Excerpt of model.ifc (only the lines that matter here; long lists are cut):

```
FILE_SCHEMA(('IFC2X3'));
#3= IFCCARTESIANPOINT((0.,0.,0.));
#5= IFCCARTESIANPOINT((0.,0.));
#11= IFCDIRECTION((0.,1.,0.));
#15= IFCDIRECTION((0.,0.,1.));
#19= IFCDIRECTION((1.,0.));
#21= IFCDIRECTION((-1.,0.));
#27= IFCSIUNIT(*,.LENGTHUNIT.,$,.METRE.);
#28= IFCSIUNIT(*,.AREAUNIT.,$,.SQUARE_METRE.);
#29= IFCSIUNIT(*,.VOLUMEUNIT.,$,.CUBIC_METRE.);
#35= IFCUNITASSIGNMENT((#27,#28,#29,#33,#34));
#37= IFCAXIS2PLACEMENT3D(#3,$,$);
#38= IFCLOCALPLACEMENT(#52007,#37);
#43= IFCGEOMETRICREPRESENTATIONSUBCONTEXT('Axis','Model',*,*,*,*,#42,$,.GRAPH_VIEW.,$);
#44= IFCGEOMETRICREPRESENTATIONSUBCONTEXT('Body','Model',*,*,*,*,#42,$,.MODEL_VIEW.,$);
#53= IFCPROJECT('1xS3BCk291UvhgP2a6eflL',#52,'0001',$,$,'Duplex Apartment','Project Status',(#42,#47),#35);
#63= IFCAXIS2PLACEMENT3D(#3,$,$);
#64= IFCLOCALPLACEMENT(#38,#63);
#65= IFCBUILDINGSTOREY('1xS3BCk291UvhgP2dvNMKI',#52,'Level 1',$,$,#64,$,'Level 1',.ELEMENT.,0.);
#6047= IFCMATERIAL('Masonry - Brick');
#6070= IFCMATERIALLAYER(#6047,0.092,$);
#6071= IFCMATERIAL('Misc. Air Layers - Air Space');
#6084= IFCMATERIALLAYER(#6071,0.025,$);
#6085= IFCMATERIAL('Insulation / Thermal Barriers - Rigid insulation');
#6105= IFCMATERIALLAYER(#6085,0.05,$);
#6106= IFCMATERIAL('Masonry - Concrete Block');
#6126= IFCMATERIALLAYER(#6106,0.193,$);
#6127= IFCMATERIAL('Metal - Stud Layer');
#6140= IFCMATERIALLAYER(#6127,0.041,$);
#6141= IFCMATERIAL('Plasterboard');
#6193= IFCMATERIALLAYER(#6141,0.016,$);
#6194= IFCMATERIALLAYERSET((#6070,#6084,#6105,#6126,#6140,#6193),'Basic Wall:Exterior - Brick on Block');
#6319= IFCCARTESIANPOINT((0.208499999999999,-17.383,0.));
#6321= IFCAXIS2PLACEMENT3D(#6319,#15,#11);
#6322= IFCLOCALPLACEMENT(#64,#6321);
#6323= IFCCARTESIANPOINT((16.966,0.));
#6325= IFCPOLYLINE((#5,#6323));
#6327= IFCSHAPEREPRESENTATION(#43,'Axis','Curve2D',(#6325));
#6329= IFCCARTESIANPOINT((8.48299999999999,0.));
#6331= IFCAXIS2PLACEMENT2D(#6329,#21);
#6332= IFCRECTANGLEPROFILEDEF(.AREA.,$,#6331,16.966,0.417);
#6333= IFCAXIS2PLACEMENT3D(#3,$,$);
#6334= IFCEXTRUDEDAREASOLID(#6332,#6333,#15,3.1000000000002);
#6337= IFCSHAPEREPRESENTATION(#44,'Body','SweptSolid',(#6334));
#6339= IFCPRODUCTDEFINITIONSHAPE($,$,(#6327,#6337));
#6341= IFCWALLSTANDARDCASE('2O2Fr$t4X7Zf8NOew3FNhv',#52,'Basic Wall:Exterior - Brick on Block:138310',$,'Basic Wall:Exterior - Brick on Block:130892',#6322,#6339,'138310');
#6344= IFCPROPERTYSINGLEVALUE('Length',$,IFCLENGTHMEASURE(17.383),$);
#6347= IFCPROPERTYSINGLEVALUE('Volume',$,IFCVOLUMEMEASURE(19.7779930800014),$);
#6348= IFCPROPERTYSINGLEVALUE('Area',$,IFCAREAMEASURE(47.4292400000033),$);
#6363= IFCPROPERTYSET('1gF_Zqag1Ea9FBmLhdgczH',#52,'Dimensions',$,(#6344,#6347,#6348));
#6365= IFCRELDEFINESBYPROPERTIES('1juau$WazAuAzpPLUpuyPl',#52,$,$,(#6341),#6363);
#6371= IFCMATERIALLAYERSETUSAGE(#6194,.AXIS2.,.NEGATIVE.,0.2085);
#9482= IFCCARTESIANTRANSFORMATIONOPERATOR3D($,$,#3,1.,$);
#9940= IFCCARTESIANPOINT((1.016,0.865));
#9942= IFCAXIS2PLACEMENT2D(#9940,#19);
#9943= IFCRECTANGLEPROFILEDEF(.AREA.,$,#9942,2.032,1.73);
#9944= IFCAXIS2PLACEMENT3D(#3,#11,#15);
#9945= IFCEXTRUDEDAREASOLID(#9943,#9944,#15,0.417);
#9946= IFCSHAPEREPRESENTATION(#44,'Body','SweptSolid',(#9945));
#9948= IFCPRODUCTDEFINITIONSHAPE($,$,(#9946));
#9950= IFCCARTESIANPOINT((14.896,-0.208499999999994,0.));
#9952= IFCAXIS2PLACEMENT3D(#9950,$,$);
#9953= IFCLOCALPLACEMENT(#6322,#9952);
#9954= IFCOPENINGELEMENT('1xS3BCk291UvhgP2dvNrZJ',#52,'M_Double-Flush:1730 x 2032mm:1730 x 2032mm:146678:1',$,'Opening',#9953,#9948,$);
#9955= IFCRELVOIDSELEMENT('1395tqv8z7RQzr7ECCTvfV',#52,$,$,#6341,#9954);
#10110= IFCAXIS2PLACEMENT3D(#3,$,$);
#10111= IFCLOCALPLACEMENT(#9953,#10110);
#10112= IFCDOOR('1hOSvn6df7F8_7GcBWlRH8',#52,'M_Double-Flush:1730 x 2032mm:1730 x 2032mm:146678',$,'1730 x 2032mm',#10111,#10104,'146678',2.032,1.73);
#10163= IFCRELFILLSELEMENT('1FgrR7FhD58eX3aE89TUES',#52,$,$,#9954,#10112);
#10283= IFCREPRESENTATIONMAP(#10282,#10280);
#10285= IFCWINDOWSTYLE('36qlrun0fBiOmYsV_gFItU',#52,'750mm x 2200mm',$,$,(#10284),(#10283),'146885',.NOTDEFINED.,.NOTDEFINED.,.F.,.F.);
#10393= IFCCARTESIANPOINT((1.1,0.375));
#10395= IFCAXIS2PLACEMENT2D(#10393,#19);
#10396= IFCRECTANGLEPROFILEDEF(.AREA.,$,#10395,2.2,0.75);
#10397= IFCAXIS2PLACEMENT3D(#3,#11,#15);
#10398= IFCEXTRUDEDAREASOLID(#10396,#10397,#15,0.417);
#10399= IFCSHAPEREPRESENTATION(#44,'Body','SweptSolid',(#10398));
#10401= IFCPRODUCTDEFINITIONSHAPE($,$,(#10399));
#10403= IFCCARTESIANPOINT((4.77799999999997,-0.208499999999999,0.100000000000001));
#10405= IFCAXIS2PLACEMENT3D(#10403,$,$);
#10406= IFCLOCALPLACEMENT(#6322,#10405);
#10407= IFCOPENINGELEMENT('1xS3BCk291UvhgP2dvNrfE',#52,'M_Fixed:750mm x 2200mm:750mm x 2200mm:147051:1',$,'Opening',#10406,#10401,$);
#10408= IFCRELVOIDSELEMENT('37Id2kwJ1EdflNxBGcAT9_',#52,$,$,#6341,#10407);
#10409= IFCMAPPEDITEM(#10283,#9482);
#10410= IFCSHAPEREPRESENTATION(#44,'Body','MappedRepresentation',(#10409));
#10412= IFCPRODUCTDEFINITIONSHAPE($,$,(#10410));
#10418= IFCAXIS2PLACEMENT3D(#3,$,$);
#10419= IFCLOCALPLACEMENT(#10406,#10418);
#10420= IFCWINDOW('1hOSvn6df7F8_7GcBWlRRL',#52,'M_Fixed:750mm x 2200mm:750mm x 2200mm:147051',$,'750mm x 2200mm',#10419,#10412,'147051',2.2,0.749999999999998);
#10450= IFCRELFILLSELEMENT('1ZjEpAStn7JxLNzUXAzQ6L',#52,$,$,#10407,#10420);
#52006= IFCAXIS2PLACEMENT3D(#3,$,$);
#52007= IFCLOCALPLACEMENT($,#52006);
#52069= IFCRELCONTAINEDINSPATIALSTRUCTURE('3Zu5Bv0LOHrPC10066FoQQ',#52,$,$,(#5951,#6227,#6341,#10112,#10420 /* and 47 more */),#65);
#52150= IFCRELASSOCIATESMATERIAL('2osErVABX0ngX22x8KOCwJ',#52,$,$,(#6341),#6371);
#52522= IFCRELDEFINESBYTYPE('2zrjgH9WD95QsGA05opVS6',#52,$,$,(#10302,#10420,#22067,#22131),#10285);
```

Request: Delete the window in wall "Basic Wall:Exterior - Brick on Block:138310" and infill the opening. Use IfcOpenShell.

```python
import ifcopenshell
import ifcopenshell.api.feature
import ifcopenshell.api.pset
import ifcopenshell.api.root
import ifcopenshell.geom
import ifcopenshell.util.element
import ifcopenshell.util.shape
import ifcopenshell.util.unit

model = ifcopenshell.open("model.ifc")
area_scale = ifcopenshell.util.unit.calculate_unit_scale(model, "AREAUNIT")
volume_scale = ifcopenshell.util.unit.calculate_unit_scale(model, "VOLUMEUNIT")
settings = ifcopenshell.geom.settings()


def volume(element):
    """Net volume in cubic metres, openings subtracted."""
    shape = ifcopenshell.geom.create_shape(settings, element)
    return ifcopenshell.util.shape.get_volume(shape.geometry)


window = model.by_id(10420)
opening = window.FillsVoids[0].RelatingOpeningElement
wall = opening.VoidsElements[0].RelatingBuildingElement
before = volume(wall)

ifcopenshell.api.root.remove_product(model, product=window)
ifcopenshell.api.feature.remove_feature(model, feature=opening)

after = volume(wall)
thickness = 0.417  # wall thickness in metres

# Update the wall's stored quantities.
pset = model.by_id(ifcopenshell.util.element.get_pset(wall, "Dimensions", should_inherit=False)["id"])
ifcopenshell.api.pset.edit_pset(model, pset=pset, properties={
    "Volume": model.create_entity("IfcVolumeMeasure", after / volume_scale),
    "Area": model.create_entity("IfcAreaMeasure", after / thickness / area_scale),
})

print(f"wall volume {before:.3f} -> {after:.3f} m3")

model.write("model_v2.ifc")
```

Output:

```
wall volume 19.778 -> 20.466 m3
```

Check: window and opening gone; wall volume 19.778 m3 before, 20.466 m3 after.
